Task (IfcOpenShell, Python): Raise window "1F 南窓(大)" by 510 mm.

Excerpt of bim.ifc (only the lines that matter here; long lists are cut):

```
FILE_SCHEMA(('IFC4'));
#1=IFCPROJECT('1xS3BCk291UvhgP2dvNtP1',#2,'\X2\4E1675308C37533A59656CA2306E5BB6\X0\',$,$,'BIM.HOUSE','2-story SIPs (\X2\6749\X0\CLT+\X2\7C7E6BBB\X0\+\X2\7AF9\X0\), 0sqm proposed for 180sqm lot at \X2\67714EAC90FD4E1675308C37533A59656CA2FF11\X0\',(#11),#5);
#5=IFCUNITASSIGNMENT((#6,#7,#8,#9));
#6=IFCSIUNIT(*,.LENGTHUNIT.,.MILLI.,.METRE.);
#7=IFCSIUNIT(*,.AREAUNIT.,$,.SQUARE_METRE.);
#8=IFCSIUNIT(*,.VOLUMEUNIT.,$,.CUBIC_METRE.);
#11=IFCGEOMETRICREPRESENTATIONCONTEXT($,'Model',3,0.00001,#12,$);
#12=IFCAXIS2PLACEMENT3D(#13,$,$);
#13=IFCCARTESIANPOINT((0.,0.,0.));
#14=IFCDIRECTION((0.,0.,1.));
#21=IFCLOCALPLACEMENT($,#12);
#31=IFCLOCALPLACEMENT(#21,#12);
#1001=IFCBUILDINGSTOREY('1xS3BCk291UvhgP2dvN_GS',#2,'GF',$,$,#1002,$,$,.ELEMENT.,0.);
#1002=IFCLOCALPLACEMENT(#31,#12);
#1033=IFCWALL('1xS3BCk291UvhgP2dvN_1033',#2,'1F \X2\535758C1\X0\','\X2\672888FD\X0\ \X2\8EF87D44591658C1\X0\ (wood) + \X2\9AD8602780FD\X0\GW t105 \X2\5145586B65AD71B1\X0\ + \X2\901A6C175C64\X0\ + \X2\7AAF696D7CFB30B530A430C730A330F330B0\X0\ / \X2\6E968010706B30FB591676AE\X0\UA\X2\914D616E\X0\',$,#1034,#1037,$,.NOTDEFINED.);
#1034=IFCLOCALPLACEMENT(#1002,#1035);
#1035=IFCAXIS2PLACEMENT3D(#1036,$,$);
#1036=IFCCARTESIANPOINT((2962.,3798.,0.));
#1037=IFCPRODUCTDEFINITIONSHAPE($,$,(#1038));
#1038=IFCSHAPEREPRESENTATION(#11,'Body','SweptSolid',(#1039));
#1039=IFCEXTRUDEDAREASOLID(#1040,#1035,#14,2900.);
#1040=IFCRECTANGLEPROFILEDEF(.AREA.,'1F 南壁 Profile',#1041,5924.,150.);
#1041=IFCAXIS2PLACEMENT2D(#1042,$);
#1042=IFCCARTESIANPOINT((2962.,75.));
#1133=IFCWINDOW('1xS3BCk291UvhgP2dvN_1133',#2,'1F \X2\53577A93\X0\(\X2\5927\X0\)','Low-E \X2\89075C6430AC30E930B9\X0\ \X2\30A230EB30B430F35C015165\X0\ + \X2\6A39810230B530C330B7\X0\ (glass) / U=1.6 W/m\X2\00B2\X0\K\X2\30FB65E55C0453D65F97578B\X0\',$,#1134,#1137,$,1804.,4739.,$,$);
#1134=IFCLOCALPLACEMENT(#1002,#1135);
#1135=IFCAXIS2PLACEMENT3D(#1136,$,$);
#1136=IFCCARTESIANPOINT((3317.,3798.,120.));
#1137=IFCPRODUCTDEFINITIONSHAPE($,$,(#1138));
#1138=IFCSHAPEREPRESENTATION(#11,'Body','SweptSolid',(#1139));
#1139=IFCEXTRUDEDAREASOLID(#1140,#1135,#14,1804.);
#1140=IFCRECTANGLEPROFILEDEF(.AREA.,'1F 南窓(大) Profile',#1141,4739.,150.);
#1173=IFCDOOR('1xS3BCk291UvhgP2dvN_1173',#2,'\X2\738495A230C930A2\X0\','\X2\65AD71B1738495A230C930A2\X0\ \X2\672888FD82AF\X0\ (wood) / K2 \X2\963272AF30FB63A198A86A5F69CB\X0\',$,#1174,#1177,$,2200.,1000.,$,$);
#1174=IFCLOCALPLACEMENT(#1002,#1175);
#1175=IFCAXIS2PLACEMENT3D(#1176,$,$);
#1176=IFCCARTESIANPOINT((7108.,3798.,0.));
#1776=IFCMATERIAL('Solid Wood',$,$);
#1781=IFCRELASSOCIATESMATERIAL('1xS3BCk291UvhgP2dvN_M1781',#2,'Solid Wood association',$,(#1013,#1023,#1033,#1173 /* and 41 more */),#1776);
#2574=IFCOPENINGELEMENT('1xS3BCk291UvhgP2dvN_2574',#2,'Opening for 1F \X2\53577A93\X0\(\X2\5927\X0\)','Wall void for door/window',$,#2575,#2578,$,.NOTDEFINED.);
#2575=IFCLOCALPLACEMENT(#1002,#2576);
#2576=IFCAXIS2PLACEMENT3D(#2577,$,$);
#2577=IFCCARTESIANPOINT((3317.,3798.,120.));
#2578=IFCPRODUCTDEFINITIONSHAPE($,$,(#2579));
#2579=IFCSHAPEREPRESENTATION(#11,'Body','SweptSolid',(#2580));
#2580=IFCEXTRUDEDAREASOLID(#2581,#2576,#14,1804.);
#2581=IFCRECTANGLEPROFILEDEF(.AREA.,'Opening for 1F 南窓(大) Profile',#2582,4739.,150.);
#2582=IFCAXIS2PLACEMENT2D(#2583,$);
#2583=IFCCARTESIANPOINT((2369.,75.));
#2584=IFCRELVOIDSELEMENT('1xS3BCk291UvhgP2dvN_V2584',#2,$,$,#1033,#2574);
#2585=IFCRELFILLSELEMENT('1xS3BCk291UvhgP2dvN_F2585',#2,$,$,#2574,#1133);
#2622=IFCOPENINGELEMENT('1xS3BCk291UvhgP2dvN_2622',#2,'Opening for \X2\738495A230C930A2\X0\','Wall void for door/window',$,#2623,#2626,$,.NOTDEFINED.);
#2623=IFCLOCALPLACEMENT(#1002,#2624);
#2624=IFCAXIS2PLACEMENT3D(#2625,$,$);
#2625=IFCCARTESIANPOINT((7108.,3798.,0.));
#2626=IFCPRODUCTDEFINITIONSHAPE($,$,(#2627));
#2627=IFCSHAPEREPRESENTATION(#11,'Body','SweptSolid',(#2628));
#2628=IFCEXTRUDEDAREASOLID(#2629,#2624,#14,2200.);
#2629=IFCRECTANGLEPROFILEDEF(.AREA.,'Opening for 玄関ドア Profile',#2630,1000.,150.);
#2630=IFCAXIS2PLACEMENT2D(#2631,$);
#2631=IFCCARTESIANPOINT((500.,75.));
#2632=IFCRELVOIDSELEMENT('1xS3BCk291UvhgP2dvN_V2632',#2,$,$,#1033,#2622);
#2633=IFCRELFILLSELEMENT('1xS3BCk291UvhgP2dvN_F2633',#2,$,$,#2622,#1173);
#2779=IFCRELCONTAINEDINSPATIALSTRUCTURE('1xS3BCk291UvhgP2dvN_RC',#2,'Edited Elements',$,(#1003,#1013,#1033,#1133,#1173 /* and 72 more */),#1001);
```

```python
import numpy as np
import ifcopenshell
import ifcopenshell.api.geometry
import ifcopenshell.util.placement
import ifcopenshell.util.unit

model = ifcopenshell.open("bim.ifc")
unit_scale = ifcopenshell.util.unit.calculate_unit_scale(model)

window = model.by_guid("1xS3BCk291UvhgP2dvN_1133")
opening = window.FillsVoids[0].RelatingOpeningElement
dz = 510.0

shift = np.array([0.0, 0.0, dz])
# The window is not placed relative to its opening, so move both.
for product in (opening, window):
    matrix = ifcopenshell.util.placement.get_local_placement(product.ObjectPlacement)
    matrix[:3, 3] += shift
    ifcopenshell.api.geometry.edit_object_placement(model, product=product, matrix=matrix, is_si=False)

print(f"moved by {dz * unit_scale:+.3f} m")

model.write("bim_edited.ifc")
```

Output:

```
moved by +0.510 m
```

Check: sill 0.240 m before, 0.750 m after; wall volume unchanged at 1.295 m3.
